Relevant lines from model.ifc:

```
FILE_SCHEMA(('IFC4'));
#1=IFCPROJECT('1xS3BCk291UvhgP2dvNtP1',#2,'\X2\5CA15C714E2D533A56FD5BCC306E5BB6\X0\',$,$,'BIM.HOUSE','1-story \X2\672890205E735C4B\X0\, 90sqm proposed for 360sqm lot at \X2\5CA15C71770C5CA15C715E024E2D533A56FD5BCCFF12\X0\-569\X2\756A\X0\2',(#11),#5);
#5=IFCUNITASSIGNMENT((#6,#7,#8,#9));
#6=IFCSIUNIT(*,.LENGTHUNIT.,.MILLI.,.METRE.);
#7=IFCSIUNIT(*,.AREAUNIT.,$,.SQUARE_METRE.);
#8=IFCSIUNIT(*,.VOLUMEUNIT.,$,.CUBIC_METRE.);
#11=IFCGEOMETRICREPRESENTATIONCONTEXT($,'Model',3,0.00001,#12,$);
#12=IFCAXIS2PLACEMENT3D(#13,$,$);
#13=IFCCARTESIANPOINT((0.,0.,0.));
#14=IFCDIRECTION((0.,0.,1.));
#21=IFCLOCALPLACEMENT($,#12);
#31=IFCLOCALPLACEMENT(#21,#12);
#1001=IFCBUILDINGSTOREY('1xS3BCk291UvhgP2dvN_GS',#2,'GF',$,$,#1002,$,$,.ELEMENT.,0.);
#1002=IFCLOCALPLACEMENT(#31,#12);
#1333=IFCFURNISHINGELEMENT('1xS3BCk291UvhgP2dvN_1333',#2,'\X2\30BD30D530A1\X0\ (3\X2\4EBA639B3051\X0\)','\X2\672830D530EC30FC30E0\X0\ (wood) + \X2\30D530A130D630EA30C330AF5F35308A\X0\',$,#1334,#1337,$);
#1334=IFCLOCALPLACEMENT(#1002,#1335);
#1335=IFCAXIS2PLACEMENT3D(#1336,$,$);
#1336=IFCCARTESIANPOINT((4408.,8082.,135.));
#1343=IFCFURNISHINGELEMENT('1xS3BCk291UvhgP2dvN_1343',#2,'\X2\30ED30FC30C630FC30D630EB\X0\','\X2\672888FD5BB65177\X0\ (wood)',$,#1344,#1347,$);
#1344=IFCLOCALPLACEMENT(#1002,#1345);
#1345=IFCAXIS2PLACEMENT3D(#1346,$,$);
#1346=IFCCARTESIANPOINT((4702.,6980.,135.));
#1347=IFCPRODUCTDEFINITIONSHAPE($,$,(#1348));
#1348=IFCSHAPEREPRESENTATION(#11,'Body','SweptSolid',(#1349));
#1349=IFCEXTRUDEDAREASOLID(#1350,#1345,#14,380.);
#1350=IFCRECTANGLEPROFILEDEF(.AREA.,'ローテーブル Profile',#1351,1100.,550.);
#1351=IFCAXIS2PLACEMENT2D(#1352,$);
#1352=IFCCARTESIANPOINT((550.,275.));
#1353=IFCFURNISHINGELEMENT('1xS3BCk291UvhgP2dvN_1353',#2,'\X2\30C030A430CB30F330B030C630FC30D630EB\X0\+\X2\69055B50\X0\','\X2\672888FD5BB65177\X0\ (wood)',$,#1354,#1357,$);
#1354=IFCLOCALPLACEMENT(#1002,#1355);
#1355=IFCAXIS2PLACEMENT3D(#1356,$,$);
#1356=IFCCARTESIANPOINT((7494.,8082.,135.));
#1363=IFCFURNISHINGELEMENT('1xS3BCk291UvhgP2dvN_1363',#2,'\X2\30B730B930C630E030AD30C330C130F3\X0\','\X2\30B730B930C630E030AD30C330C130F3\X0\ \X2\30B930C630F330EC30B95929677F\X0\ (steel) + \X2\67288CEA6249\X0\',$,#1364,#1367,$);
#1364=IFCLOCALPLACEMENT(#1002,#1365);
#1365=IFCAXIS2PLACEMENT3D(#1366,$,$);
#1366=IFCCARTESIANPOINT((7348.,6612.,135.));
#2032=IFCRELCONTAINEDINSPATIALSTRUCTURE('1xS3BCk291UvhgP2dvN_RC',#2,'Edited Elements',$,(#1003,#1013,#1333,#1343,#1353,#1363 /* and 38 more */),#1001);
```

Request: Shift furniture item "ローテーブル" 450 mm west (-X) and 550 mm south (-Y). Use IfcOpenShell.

```python
import ifcopenshell
import ifcopenshell.api.geometry
import ifcopenshell.util.placement
import ifcopenshell.util.unit

model = ifcopenshell.open("model.ifc")
unit_scale = ifcopenshell.util.unit.calculate_unit_scale(model)

item = model.by_guid("1xS3BCk291UvhgP2dvN_1343")
matrix = ifcopenshell.util.placement.get_local_placement(item.ObjectPlacement)
matrix[0, 3] -= 0.45 / unit_scale
matrix[1, 3] -= 0.55 / unit_scale
ifcopenshell.api.geometry.edit_object_placement(model, product=item, matrix=matrix, is_si=False)

print(ifcopenshell.util.placement.get_local_placement(item.ObjectPlacement).round(3) + 0.0)

model.write("model_rev.ifc")
```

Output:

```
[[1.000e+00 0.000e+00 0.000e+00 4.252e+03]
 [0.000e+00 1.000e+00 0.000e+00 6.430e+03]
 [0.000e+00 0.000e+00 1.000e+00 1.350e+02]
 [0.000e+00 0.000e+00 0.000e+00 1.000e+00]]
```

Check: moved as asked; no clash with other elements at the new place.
